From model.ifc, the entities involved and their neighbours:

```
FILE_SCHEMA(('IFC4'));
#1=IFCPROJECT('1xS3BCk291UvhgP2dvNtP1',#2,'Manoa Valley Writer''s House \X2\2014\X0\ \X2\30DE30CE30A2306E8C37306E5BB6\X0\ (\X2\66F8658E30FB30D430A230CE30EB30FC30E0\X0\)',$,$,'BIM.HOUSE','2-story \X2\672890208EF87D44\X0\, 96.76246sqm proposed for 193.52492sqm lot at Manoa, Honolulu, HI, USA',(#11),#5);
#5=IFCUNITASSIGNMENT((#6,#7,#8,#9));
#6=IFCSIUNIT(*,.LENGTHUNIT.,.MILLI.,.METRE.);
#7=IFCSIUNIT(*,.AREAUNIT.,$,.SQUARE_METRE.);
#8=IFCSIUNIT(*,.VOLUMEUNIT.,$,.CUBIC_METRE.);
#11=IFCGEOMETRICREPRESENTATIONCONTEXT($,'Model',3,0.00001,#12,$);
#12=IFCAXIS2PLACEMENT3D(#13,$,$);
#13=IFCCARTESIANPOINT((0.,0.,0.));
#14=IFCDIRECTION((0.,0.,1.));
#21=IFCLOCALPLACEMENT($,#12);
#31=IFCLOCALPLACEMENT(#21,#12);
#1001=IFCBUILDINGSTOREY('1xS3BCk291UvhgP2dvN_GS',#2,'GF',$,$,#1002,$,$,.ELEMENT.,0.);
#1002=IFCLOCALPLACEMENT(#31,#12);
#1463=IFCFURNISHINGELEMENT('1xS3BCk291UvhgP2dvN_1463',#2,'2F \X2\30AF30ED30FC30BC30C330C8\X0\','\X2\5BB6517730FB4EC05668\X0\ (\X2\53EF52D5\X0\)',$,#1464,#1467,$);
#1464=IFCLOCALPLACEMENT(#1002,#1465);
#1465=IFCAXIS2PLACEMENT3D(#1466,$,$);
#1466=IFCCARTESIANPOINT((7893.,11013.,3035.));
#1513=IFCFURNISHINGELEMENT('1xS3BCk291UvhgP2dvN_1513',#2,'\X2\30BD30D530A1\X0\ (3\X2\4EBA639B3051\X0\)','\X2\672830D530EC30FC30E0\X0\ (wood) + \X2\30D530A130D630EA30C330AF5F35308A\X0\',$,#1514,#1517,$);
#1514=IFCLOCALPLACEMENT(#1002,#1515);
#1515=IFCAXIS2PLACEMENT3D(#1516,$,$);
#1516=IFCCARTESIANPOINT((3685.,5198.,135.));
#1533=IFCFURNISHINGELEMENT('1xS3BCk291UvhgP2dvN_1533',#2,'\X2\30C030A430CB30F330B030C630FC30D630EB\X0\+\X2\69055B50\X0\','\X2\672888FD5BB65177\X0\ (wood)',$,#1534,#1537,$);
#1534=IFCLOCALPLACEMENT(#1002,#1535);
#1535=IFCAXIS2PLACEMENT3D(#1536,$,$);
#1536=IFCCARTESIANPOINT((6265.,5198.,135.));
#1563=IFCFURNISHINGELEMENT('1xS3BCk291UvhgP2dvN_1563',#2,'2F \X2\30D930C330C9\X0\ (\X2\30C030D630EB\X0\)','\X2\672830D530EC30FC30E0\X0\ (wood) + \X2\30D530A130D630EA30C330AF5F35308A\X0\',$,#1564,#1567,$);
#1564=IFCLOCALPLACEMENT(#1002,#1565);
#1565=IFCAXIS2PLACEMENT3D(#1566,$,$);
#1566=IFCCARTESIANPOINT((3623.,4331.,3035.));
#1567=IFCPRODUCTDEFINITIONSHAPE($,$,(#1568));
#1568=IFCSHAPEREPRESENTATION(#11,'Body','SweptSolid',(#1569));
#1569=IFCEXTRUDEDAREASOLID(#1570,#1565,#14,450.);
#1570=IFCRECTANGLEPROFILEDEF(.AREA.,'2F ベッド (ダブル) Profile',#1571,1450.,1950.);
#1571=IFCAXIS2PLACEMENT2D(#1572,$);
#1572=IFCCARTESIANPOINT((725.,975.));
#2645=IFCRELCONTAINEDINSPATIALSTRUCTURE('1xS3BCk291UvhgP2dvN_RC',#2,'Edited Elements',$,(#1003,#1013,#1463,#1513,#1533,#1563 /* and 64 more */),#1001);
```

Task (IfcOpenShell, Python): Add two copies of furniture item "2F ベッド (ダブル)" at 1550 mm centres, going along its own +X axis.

```python
import ifcopenshell
import ifcopenshell.api.geometry
import ifcopenshell.api.root
import ifcopenshell.util.element
import ifcopenshell.util.placement

model = ifcopenshell.open("model.ifc")


def reuse_history(source, copy):
    """copy_class also copies each property set's owner history, people and application; keep the originals."""
    for rel in copy.IsDefinedBy:
        if rel.is_a("IfcRelDefinesByProperties") and (history := rel.RelatingPropertyDefinition.OwnerHistory):
            rel.RelatingPropertyDefinition.OwnerHistory = source.OwnerHistory
            ifcopenshell.util.element.remove_deep2(model, history)


source = model.by_guid("1xS3BCk291UvhgP2dvN_1563")
base = ifcopenshell.util.placement.get_local_placement(source.ObjectPlacement)
step = base[:3, 0] * 1550.0

for i in range(1, 3):
    copy = ifcopenshell.api.root.copy_class(model, product=source)
    copy.Representation = ifcopenshell.util.element.copy_deep(
        model, source.Representation, exclude=["IfcGeometricRepresentationContext", "IfcRepresentationMap"]
    )
    reuse_history(source, copy)
    matrix = base.copy()
    matrix[:3, 3] += i * step
    print("added at", matrix[:3, 3].round(3) + 0.0)
    ifcopenshell.api.geometry.edit_object_placement(model, product=copy, matrix=matrix, is_si=False)

model.write("model_rev.ifc")
```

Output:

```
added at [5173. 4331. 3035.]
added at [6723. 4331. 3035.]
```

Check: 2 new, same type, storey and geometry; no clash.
